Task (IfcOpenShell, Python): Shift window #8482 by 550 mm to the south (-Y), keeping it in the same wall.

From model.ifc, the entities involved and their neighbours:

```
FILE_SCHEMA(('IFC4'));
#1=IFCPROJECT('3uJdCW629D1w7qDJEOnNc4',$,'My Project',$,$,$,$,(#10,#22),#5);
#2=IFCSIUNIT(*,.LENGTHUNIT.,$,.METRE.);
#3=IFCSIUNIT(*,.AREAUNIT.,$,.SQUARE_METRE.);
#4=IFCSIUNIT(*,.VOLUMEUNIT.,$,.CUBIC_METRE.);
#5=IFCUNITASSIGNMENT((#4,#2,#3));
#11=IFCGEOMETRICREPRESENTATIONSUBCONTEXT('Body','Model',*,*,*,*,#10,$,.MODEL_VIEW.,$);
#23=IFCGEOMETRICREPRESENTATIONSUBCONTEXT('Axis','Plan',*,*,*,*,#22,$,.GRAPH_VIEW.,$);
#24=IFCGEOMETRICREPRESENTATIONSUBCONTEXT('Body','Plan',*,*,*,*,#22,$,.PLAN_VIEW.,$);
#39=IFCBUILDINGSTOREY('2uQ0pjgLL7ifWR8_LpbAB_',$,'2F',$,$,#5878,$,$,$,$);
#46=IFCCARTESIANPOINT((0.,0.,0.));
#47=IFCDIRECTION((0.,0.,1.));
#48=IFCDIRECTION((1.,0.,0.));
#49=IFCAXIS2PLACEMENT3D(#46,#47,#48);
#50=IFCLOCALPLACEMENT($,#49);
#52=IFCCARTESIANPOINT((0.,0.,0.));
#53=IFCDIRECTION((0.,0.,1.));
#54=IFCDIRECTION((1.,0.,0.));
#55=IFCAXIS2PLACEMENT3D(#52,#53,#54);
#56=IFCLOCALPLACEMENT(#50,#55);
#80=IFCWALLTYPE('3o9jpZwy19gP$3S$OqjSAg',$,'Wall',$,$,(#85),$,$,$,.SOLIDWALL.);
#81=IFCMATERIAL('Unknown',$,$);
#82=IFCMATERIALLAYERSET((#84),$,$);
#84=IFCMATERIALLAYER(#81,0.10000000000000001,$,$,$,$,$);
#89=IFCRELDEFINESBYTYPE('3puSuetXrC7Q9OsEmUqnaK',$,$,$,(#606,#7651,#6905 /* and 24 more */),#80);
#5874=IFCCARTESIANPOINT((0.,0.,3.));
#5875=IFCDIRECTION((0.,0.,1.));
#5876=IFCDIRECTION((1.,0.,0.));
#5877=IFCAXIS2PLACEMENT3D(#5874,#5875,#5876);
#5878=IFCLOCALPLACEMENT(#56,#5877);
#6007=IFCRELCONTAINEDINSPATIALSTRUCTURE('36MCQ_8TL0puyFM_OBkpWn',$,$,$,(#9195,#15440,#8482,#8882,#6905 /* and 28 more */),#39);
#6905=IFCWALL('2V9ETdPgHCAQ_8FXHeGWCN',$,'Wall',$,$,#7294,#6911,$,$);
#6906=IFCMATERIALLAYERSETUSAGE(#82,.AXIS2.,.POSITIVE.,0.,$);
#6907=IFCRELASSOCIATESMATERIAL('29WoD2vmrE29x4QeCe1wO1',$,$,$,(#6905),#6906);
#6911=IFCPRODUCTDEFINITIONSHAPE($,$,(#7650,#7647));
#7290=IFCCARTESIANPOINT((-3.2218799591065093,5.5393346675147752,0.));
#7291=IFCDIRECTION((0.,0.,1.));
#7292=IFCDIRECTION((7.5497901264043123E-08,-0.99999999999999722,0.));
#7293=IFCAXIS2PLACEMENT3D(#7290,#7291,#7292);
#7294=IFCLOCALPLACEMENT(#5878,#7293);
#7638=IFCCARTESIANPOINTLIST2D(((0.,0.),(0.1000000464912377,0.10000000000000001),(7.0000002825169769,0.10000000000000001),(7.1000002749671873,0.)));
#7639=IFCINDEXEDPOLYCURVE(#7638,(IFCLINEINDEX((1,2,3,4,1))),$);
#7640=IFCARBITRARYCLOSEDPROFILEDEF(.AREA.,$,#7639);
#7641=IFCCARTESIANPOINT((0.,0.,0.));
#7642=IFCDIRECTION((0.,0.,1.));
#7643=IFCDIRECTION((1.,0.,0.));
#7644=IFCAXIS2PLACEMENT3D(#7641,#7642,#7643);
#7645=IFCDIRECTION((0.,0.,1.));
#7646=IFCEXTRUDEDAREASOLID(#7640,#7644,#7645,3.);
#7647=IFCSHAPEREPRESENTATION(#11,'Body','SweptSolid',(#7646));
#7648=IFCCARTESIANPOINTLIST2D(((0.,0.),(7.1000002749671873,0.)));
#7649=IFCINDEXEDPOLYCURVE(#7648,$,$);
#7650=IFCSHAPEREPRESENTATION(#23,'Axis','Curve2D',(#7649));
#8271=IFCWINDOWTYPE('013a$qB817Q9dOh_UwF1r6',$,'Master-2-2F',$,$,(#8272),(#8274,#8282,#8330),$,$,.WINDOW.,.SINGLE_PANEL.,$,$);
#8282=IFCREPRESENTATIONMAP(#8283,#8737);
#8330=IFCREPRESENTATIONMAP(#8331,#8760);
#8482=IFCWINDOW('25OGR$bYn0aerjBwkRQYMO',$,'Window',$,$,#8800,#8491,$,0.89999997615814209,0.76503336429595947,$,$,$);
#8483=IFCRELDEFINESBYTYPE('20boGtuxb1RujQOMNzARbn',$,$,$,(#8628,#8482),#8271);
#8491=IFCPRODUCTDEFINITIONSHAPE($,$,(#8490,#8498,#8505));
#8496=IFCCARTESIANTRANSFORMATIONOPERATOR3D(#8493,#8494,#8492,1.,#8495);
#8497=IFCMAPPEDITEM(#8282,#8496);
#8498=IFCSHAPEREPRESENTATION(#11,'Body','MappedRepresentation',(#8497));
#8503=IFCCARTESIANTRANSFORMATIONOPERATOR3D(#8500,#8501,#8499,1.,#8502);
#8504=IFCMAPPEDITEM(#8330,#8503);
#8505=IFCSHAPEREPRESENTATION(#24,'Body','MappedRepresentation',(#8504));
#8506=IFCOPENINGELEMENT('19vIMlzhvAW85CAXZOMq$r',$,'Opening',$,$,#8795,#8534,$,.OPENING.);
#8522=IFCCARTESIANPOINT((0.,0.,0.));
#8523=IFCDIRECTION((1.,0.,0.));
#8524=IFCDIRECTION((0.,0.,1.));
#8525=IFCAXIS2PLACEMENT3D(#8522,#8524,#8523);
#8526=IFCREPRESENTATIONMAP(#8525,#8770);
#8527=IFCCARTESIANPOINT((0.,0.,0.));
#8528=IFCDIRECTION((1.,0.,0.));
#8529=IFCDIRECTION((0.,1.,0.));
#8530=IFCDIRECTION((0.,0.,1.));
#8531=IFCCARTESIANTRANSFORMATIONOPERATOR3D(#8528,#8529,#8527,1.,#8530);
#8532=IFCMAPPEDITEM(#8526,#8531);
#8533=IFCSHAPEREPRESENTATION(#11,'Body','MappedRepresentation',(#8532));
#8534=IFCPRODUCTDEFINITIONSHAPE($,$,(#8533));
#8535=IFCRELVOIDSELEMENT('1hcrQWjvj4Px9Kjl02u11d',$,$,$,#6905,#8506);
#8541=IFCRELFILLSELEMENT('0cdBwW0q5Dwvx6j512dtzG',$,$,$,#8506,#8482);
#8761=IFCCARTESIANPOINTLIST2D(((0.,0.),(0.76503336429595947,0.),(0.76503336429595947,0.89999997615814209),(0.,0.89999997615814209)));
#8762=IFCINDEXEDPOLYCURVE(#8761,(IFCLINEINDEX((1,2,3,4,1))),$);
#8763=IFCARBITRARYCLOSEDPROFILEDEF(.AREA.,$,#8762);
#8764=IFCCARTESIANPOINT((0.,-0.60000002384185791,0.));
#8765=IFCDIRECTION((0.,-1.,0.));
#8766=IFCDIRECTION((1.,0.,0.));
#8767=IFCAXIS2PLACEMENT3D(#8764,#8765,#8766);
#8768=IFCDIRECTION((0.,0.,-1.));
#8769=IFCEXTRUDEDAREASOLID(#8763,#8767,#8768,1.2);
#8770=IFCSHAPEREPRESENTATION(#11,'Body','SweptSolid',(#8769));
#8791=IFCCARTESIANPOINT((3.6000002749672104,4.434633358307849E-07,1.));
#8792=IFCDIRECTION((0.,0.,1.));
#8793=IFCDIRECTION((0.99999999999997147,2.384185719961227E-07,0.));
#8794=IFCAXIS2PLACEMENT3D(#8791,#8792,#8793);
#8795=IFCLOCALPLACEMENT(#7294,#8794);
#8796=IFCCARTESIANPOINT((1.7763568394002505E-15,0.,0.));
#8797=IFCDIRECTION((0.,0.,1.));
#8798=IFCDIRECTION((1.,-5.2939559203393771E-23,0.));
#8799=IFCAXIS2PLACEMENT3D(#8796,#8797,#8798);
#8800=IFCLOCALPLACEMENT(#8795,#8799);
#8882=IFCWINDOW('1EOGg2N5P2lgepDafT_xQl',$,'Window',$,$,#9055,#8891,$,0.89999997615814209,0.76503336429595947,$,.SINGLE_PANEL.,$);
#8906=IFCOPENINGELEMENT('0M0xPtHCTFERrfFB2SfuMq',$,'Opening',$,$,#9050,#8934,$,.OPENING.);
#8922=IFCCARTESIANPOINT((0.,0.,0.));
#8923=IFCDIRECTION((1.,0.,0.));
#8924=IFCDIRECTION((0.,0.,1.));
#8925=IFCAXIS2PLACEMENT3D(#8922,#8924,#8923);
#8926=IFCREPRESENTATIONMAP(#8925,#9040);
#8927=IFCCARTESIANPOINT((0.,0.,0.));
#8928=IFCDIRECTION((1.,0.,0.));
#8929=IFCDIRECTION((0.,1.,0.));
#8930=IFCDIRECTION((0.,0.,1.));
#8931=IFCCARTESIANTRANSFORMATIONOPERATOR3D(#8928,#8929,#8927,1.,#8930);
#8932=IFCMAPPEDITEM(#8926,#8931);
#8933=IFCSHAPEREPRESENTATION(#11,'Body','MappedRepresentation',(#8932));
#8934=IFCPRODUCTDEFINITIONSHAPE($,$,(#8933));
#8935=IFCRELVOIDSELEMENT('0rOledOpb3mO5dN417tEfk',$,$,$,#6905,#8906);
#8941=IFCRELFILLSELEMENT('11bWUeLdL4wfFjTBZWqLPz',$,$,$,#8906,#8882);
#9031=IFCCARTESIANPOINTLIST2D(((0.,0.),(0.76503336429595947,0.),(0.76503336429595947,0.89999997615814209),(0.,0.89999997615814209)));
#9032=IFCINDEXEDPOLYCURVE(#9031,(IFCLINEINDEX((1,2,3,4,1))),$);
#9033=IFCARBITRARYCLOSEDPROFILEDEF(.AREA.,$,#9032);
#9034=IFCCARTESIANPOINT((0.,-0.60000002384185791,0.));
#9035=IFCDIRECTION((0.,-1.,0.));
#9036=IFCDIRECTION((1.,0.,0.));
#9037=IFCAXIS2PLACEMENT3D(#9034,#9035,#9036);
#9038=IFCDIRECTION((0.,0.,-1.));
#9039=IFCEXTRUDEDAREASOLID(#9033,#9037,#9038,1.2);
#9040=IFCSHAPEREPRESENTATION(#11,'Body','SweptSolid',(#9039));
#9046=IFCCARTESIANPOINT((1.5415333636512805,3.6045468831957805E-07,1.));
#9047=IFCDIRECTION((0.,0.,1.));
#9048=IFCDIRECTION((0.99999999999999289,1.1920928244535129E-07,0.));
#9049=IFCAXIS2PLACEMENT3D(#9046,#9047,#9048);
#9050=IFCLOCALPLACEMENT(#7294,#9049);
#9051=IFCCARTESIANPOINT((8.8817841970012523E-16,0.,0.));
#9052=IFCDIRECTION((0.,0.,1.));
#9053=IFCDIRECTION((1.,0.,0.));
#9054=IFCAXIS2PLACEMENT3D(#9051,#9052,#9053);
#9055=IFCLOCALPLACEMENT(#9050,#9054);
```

```python
import ifcopenshell
import ifcopenshell.api.geometry
import ifcopenshell.util.placement

model = ifcopenshell.open("model.ifc")

window = model.by_guid("25OGR$bYn0aerjBwkRQYMO")
opening = window.FillsVoids[0].RelatingOpeningElement
wall = opening.VoidsElements[0].RelatingBuildingElement

wall_matrix = ifcopenshell.util.placement.get_local_placement(wall.ObjectPlacement)
shift = wall_matrix[:3, 0] * 0.55
before = ifcopenshell.util.placement.get_local_placement(window.ObjectPlacement)[:3, 3].copy()

# The window is placed relative to its opening, so it follows when the opening moves.
matrix = ifcopenshell.util.placement.get_local_placement(opening.ObjectPlacement)
matrix[:3, 3] += shift
ifcopenshell.api.geometry.edit_object_placement(
    model, product=opening, matrix=matrix, is_si=False, should_transform_children=True
)

after = ifcopenshell.util.placement.get_local_placement(window.ObjectPlacement)[:3, 3]
print("window moved by", (after - before).round(3) + 0.0)

model.write("model_v2.ifc")
```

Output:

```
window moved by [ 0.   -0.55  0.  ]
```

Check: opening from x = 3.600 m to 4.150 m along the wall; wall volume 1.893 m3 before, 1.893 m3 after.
